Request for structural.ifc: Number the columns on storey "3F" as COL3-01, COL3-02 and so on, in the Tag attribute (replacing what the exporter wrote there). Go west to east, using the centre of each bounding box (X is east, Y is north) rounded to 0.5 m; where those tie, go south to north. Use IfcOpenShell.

First a look at what the model holds.

```python
import ifcopenshell
import ifcopenshell.util.element
import ifcopenshell.util.placement

model = ifcopenshell.open("structural.ifc")
print(model.schema)
storey = next(s for s in model.by_type("IfcBuildingStorey") if s.Name == "3F")
columns = [e for e in ifcopenshell.util.element.get_decomposition(storey) if e.is_a("IfcColumn")]
for e in sorted(columns, key=lambda e: e.id()):
    origin = ifcopenshell.util.placement.get_local_placement(e.ObjectPlacement)[:3, 3]
    print(e.id(), e.Tag, e.Name, origin.round(2) + 0.0, sep=" | ")
```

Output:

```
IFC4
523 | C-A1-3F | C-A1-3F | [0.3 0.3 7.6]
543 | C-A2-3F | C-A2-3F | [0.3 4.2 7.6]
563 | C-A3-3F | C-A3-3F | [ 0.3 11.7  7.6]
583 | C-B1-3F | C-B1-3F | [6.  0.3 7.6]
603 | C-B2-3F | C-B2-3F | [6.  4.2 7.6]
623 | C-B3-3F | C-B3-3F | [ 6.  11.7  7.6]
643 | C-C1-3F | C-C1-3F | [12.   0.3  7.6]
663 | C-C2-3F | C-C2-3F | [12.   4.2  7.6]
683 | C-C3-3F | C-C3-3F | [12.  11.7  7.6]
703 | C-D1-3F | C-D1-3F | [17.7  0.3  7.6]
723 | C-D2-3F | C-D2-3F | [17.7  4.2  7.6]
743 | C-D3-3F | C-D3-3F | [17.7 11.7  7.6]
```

```python
import ifcopenshell
import ifcopenshell.geom
import ifcopenshell.util.element
import ifcopenshell.util.shape

model = ifcopenshell.open("structural.ifc")
settings = ifcopenshell.geom.settings()
settings.set("use-world-coords", True)


def centre(element):
    shape = ifcopenshell.geom.create_shape(settings, element)
    return ifcopenshell.util.shape.get_bbox_centroid(shape.geometry)


storey = next(s for s in model.by_type("IfcBuildingStorey") if s.Name == "3F")
columns = [e for e in ifcopenshell.util.element.get_decomposition(storey) if e.is_a("IfcColumn")]

# Insertion points can sit at a corner or the storey origin, so sort by the geometry (in metres).
centres = {e: centre(e) for e in columns}
columns.sort(key=lambda e: (round(centres[e][0] / 0.5), centres[e][1]))

for i, e in enumerate(columns, start=1):
    number = f"COL3-{i:02d}"
    e.Tag = number
    print(e.id(), number)

model.write("structural_updated.ifc")
```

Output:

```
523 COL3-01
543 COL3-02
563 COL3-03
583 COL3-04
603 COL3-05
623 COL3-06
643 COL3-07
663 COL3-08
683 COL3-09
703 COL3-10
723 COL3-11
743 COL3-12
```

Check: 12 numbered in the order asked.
